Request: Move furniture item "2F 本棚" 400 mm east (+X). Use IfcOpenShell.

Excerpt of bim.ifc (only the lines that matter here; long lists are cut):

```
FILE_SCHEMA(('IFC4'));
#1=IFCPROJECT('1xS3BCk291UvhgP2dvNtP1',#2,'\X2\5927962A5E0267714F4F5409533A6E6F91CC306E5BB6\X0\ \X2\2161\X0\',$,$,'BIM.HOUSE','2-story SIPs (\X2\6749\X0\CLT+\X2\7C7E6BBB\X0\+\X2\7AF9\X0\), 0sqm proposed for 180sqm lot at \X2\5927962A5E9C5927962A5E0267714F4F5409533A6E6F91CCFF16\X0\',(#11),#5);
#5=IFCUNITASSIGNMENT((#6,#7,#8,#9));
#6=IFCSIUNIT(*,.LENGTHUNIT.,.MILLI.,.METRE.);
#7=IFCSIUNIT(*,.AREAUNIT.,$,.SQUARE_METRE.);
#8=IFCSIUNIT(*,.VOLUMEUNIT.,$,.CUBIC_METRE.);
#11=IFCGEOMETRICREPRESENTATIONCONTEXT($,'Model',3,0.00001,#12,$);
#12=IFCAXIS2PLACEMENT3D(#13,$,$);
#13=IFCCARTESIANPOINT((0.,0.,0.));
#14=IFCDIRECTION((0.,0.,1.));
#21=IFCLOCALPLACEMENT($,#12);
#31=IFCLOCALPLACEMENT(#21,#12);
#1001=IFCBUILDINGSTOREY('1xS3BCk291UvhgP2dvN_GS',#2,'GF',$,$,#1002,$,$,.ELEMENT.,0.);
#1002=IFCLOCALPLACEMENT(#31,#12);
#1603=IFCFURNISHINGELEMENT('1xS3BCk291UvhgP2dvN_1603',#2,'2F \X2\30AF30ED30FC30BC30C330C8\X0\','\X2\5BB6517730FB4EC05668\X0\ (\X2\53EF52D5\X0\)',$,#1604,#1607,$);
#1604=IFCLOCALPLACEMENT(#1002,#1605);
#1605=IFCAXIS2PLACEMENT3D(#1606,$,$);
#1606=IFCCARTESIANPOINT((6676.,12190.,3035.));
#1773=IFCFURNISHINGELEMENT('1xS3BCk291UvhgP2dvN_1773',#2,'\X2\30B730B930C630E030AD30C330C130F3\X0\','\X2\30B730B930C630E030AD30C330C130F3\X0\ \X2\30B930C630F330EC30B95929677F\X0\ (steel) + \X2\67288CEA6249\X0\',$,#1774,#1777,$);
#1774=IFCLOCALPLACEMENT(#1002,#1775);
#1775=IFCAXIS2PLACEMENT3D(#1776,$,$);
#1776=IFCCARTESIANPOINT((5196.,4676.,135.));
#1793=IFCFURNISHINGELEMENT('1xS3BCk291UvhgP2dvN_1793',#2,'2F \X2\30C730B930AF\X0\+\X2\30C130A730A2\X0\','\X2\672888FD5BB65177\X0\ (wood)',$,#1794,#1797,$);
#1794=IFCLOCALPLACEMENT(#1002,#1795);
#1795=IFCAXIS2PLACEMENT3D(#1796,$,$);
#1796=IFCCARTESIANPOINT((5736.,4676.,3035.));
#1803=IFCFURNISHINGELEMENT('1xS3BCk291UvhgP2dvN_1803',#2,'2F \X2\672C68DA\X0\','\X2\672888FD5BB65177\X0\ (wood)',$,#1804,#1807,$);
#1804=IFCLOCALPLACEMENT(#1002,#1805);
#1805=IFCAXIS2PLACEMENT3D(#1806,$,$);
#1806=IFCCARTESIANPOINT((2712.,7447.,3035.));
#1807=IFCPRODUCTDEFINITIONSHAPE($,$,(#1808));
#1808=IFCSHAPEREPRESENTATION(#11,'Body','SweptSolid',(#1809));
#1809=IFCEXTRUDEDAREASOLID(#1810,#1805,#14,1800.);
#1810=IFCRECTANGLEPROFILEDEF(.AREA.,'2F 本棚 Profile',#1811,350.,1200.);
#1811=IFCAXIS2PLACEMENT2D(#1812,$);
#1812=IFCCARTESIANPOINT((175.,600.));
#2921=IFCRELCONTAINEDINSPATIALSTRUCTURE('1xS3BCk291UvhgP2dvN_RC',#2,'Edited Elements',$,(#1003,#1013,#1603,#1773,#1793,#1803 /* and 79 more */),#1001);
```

```python
import ifcopenshell
import ifcopenshell.api.geometry
import ifcopenshell.util.placement

model = ifcopenshell.open("bim.ifc")

item = model.by_id(1803)
matrix = ifcopenshell.util.placement.get_local_placement(item.ObjectPlacement)
matrix[0, 3] += 400.0
ifcopenshell.api.geometry.edit_object_placement(model, product=item, matrix=matrix, is_si=False)

print(ifcopenshell.util.placement.get_local_placement(item.ObjectPlacement).round(3) + 0.0)

model.write("bim_updated.ifc")
```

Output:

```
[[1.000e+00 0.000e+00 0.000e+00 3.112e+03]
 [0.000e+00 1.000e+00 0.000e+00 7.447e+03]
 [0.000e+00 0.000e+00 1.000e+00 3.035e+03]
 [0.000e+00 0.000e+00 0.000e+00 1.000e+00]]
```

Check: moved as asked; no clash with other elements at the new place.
